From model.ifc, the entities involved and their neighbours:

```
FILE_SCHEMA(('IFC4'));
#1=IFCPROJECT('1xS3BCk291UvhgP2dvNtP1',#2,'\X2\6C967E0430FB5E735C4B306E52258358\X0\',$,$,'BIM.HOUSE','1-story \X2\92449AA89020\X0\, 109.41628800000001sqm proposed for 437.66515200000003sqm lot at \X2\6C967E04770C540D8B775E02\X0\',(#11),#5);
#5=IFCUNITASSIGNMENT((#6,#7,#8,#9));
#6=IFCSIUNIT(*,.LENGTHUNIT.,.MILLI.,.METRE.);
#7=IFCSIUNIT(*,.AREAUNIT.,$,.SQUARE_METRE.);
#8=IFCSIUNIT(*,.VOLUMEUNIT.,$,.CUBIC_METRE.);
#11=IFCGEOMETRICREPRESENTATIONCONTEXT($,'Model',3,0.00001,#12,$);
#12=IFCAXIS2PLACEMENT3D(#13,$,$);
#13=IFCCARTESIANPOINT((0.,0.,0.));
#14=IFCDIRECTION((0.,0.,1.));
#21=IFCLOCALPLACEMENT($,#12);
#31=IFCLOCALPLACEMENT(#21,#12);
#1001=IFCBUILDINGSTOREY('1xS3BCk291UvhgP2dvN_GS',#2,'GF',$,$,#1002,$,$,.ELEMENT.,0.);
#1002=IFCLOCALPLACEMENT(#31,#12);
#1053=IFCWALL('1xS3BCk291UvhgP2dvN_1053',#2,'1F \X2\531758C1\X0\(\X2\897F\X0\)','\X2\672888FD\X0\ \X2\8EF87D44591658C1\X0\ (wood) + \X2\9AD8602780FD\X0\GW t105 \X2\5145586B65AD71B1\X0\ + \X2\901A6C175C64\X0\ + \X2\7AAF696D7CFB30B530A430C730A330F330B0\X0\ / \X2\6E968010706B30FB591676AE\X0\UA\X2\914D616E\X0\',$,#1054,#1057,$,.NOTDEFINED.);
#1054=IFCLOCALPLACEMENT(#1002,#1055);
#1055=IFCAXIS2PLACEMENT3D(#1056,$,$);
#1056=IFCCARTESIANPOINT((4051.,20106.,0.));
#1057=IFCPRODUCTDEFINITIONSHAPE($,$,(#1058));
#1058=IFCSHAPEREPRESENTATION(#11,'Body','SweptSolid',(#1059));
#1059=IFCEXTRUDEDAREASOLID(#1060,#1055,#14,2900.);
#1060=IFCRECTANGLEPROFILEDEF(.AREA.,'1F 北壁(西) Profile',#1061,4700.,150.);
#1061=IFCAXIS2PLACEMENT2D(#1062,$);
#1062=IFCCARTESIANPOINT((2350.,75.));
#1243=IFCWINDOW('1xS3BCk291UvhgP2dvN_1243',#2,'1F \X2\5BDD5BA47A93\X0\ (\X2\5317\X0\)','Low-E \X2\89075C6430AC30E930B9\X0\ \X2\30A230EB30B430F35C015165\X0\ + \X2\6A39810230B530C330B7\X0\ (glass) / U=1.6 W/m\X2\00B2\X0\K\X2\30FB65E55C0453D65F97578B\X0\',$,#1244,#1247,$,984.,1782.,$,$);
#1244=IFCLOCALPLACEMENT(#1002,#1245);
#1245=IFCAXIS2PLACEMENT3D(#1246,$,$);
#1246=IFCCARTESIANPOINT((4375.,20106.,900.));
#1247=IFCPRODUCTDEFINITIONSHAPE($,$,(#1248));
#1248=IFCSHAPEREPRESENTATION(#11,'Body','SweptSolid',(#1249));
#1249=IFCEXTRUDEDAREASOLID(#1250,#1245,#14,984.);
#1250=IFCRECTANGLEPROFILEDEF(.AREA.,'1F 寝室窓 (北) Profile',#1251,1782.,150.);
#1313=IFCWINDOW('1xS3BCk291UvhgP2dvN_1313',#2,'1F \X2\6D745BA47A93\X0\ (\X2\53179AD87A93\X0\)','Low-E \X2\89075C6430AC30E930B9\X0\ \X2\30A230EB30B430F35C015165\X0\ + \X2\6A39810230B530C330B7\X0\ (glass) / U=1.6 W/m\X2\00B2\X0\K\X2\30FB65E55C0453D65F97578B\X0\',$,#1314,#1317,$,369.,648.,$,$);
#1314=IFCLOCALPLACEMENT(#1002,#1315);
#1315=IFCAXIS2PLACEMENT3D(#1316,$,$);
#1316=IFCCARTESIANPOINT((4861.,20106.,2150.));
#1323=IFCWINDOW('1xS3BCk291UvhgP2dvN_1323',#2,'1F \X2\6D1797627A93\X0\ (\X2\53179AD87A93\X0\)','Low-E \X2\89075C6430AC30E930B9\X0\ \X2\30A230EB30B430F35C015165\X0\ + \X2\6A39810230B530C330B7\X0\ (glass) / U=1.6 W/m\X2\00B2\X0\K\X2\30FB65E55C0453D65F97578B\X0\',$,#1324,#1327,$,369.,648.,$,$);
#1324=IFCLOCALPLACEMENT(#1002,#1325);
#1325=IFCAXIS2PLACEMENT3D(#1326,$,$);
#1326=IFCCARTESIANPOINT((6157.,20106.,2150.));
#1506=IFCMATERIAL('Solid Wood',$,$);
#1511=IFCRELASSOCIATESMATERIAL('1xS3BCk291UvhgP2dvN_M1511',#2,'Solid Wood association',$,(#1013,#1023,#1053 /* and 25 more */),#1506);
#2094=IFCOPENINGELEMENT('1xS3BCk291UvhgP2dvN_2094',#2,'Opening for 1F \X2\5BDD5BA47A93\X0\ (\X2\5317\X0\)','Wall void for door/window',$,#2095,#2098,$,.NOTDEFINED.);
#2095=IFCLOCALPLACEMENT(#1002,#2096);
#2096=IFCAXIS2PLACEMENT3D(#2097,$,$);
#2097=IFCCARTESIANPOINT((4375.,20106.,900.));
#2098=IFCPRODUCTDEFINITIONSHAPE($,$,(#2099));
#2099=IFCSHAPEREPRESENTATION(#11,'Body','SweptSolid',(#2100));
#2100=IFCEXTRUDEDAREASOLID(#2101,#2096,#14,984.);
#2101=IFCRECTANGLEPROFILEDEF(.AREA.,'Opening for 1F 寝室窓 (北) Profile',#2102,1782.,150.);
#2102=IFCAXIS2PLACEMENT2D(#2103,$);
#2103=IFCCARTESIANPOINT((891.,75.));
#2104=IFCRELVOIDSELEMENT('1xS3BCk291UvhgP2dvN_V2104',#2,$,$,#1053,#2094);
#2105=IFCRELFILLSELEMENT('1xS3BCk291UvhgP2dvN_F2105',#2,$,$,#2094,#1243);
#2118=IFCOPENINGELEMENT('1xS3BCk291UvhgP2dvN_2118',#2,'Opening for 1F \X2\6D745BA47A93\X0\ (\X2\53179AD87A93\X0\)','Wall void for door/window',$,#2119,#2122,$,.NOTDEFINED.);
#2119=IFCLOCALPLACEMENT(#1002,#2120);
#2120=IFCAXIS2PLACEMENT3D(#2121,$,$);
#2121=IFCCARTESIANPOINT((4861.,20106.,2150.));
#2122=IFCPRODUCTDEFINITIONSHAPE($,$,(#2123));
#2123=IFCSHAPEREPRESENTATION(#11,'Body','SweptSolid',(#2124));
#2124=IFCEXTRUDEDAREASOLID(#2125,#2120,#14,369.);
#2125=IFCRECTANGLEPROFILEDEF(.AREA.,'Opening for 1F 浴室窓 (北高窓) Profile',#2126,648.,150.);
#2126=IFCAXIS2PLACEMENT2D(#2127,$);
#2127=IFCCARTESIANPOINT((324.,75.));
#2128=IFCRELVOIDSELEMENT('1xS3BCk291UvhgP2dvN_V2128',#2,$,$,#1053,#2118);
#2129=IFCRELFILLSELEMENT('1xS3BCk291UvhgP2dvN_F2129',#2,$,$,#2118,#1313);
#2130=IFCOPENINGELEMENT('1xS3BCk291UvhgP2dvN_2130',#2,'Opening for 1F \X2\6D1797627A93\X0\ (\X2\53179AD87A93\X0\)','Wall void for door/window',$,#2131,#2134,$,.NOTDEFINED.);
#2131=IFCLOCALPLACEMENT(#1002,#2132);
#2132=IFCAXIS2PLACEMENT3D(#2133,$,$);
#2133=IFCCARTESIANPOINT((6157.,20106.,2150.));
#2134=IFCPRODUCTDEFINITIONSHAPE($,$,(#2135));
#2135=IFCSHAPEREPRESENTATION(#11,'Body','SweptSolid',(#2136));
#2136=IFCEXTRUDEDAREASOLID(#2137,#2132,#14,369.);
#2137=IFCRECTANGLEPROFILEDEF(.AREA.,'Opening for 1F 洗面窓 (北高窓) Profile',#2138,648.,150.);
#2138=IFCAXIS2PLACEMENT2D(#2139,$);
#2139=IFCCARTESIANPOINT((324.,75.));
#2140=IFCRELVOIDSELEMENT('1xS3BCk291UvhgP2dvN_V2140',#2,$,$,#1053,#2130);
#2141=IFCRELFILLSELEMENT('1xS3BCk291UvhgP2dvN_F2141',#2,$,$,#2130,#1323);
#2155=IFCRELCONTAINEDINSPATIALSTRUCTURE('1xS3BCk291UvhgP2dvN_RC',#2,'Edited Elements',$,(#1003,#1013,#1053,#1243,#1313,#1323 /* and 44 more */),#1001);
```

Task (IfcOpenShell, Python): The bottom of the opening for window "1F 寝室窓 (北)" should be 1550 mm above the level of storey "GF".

```python
import numpy as np
import ifcopenshell
import ifcopenshell.api.geometry
import ifcopenshell.geom
import ifcopenshell.util.element
import ifcopenshell.util.placement
import ifcopenshell.util.shape
import ifcopenshell.util.unit

model = ifcopenshell.open("model.ifc")
unit_scale = ifcopenshell.util.unit.calculate_unit_scale(model)

window = model.by_id(1243)
opening = window.FillsVoids[0].RelatingOpeningElement
storey = ifcopenshell.util.element.get_container(window, ifc_class="IfcBuildingStorey")
level = ifcopenshell.util.placement.get_local_placement(storey.ObjectPlacement)[2, 3]

# The opening's origin need not be at the sill, so measure its lowest point.
shape = ifcopenshell.geom.create_shape(ifcopenshell.geom.settings(), opening)
bottom = ifcopenshell.util.shape.get_shape_bottom_elevation(shape, shape.geometry) / unit_scale
dz = level + 1.55 / unit_scale - bottom

shift = np.array([0.0, 0.0, dz])
# The window is not placed relative to its opening, so move both.
for product in (opening, window):
    matrix = ifcopenshell.util.placement.get_local_placement(product.ObjectPlacement)
    matrix[:3, 3] += shift
    ifcopenshell.api.geometry.edit_object_placement(model, product=product, matrix=matrix, is_si=False)

print(f"moved by {dz * unit_scale:+.3f} m")

model.write("model_v2.ifc")
```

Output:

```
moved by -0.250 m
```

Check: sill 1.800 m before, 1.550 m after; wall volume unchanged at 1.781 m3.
